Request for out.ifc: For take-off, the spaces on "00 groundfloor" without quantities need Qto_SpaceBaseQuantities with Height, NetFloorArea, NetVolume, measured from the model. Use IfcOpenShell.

First a look at what the model holds.

```python
import ifcopenshell
import ifcopenshell.util.element
import ifcopenshell.util.unit

model = ifcopenshell.open("out.ifc")
print(model.schema)
for unit_type in ("LENGTHUNIT", "AREAUNIT", "VOLUMEUNIT"):
    print(unit_type, ifcopenshell.util.unit.calculate_unit_scale(model, unit_type))
storey = next(s for s in model.by_type("IfcBuildingStorey") if s.Name == "00 groundfloor")
spaces = [e for e in ifcopenshell.util.element.get_decomposition(storey) if e.is_a("IfcSpace")]
for e in sorted(spaces, key=lambda e: e.id()):
    print(e.id(), e.is_a(), e.Name, list(ifcopenshell.util.element.get_psets(e, qtos_only=True)), sep=" | ")
```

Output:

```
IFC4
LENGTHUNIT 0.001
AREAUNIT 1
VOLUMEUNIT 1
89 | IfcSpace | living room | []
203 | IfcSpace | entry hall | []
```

```python
import ifcopenshell
import ifcopenshell.api.pset
import ifcopenshell.geom
import ifcopenshell.util.element
import ifcopenshell.util.shape
import ifcopenshell.util.unit

model = ifcopenshell.open("out.ifc")
unit_scale = ifcopenshell.util.unit.calculate_unit_scale(model)
area_scale = ifcopenshell.util.unit.calculate_unit_scale(model, "AREAUNIT")
volume_scale = ifcopenshell.util.unit.calculate_unit_scale(model, "VOLUMEUNIT")
settings = ifcopenshell.geom.settings()

storey = next(s for s in model.by_type("IfcBuildingStorey") if s.Name == "00 groundfloor")
spaces = [e for e in ifcopenshell.util.element.get_decomposition(storey) if e.is_a("IfcSpace")]

for e in sorted(spaces, key=lambda e: e.id()):
    if ifcopenshell.util.element.get_psets(e, qtos_only=True, should_inherit=False):
        continue
    # Geometry comes back in metres, in the element's own axes.
    shape = ifcopenshell.geom.create_shape(settings, e)
    values = {
        "Height": ifcopenshell.util.shape.get_z(shape.geometry) / unit_scale,
        "NetFloorArea": ifcopenshell.util.shape.get_footprint_area(shape.geometry) / area_scale,
        "NetVolume": ifcopenshell.util.shape.get_volume(shape.geometry) / volume_scale,
    }
    qto = ifcopenshell.api.pset.add_qto(model, product=e, name="Qto_SpaceBaseQuantities")
    ifcopenshell.api.pset.edit_qto(model, qto=qto, properties=values)
    print(e.id(), {k: round(v, 3) for k, v in values.items()})

model.write("out-out.ifc")
```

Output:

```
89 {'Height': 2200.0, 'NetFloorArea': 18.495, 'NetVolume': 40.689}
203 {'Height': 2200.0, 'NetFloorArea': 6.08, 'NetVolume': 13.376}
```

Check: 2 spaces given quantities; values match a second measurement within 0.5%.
